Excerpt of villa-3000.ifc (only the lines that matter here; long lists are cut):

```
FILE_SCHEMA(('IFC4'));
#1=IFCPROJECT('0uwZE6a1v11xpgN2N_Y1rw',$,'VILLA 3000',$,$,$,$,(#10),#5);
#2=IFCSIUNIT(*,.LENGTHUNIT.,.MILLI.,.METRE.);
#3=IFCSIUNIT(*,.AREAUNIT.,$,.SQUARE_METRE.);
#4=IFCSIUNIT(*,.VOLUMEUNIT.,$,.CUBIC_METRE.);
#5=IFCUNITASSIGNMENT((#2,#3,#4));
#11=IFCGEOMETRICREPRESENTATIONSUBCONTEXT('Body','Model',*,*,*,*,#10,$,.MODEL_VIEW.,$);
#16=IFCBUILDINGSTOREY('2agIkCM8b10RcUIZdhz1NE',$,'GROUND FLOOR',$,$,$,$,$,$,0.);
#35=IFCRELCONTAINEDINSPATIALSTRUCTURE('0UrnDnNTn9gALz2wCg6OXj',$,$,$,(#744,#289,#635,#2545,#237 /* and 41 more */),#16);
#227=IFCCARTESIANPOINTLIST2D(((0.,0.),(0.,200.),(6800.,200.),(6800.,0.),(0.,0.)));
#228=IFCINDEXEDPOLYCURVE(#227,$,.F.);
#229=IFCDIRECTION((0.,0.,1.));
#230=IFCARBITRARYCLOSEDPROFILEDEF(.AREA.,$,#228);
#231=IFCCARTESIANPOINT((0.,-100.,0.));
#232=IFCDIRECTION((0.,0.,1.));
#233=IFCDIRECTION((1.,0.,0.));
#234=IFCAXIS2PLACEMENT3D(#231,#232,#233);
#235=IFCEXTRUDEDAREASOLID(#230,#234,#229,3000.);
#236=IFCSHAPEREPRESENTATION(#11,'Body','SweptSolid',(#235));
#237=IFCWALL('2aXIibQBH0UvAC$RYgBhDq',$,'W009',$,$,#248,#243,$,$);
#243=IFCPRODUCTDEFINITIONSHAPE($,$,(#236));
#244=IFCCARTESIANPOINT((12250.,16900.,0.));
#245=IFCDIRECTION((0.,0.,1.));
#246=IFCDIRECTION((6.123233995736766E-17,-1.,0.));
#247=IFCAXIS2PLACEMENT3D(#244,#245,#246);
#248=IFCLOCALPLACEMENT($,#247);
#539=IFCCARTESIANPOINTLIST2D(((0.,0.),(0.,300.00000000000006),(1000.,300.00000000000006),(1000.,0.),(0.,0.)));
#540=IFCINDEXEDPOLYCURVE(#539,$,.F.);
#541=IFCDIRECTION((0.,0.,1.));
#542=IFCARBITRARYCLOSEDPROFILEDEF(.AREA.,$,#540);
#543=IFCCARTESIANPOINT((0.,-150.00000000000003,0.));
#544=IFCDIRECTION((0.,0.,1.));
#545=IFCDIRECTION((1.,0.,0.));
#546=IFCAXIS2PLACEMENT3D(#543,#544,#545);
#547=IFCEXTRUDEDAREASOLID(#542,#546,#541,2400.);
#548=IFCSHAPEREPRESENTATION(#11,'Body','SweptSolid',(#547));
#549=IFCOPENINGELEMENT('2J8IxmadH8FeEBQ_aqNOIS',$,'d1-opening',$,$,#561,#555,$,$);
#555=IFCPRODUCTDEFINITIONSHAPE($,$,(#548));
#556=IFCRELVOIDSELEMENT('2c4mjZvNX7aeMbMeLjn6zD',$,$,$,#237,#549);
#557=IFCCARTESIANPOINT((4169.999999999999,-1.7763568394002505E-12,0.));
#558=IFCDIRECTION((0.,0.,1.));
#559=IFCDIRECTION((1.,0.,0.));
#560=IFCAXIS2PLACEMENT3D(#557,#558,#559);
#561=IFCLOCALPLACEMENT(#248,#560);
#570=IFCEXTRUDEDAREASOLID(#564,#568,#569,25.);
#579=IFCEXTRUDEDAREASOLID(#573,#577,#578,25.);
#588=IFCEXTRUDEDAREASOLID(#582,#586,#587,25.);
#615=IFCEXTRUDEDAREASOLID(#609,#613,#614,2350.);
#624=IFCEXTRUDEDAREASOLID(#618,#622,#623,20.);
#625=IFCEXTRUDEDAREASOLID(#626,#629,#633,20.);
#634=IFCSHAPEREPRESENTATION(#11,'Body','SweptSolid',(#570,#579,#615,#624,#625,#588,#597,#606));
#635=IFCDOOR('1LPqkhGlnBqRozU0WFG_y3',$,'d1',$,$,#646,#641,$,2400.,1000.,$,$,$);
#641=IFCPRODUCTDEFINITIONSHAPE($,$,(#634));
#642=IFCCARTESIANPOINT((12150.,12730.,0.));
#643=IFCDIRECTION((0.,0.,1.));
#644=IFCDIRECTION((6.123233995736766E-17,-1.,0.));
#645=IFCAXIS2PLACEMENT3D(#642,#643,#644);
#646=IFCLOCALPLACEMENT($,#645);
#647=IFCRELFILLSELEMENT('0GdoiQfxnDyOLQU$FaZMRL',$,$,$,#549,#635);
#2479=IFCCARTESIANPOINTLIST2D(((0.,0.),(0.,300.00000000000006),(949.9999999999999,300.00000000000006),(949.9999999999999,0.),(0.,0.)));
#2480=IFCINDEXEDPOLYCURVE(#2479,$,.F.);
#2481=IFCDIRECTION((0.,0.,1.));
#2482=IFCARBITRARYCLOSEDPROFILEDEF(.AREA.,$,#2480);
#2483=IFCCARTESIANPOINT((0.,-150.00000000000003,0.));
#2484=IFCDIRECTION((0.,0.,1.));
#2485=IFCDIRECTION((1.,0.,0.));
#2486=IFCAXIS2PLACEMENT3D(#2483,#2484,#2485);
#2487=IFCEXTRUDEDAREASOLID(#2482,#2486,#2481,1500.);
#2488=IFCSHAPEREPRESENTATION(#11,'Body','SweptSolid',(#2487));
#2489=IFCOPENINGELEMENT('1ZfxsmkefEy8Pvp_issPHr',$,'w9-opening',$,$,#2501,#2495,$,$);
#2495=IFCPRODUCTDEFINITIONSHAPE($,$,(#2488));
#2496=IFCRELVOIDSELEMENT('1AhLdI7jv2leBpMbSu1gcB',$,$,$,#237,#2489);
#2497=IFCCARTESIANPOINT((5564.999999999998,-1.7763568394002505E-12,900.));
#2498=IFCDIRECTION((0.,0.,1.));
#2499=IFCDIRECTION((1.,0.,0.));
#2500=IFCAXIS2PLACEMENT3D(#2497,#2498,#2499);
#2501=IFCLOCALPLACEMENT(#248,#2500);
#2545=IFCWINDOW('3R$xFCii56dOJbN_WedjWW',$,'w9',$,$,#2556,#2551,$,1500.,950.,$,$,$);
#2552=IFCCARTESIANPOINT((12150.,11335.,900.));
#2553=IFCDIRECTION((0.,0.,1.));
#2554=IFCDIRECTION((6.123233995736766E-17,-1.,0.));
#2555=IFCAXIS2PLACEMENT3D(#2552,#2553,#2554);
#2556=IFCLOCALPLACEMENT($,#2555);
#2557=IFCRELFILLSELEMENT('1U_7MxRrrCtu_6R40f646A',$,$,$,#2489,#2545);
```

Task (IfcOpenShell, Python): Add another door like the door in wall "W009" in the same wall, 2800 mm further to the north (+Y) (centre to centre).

```python
import ifcopenshell
import ifcopenshell.api.feature
import ifcopenshell.api.geometry
import ifcopenshell.api.root
import ifcopenshell.geom
import ifcopenshell.util.element
import ifcopenshell.util.placement
import ifcopenshell.util.shape

model = ifcopenshell.open("villa-3000.ifc")
settings = ifcopenshell.geom.settings()


def volume(element):
    """Net volume in cubic metres, openings subtracted."""
    shape = ifcopenshell.geom.create_shape(settings, element)
    return ifcopenshell.util.shape.get_volume(shape.geometry)


door = model.by_id(635)
opening = door.FillsVoids[0].RelatingOpeningElement
wall = opening.VoidsElements[0].RelatingBuildingElement
before = volume(wall)
shift = ifcopenshell.util.placement.get_local_placement(wall.ObjectPlacement)[:3, 0] * -2800.0

# copy_class copies the void relationship, type, container and properties, but no geometry.
new_opening = ifcopenshell.api.root.copy_class(model, product=opening)
new_opening.Representation = ifcopenshell.util.element.copy_deep(
    model, opening.Representation, exclude=["IfcGeometricRepresentationContext", "IfcRepresentationMap"]
)
new_door = ifcopenshell.api.root.copy_class(model, product=door)
new_door.Representation = ifcopenshell.util.element.copy_deep(
    model, door.Representation, exclude=["IfcGeometricRepresentationContext", "IfcRepresentationMap"]
)
ifcopenshell.api.feature.add_filling(model, opening=new_opening, element=new_door)

for old, new in ((opening, new_opening), (door, new_door)):
    matrix = ifcopenshell.util.placement.get_local_placement(old.ObjectPlacement)
    matrix[:3, 3] += shift
    ifcopenshell.api.geometry.edit_object_placement(model, product=new, matrix=matrix, is_si=False)

after = volume(wall)

print(f"wall volume {before:.3f} -> {after:.3f} m3")

model.write("villa-3000_rev.ifc")
```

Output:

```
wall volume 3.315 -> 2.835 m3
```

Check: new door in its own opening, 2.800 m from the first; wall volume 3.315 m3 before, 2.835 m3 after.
